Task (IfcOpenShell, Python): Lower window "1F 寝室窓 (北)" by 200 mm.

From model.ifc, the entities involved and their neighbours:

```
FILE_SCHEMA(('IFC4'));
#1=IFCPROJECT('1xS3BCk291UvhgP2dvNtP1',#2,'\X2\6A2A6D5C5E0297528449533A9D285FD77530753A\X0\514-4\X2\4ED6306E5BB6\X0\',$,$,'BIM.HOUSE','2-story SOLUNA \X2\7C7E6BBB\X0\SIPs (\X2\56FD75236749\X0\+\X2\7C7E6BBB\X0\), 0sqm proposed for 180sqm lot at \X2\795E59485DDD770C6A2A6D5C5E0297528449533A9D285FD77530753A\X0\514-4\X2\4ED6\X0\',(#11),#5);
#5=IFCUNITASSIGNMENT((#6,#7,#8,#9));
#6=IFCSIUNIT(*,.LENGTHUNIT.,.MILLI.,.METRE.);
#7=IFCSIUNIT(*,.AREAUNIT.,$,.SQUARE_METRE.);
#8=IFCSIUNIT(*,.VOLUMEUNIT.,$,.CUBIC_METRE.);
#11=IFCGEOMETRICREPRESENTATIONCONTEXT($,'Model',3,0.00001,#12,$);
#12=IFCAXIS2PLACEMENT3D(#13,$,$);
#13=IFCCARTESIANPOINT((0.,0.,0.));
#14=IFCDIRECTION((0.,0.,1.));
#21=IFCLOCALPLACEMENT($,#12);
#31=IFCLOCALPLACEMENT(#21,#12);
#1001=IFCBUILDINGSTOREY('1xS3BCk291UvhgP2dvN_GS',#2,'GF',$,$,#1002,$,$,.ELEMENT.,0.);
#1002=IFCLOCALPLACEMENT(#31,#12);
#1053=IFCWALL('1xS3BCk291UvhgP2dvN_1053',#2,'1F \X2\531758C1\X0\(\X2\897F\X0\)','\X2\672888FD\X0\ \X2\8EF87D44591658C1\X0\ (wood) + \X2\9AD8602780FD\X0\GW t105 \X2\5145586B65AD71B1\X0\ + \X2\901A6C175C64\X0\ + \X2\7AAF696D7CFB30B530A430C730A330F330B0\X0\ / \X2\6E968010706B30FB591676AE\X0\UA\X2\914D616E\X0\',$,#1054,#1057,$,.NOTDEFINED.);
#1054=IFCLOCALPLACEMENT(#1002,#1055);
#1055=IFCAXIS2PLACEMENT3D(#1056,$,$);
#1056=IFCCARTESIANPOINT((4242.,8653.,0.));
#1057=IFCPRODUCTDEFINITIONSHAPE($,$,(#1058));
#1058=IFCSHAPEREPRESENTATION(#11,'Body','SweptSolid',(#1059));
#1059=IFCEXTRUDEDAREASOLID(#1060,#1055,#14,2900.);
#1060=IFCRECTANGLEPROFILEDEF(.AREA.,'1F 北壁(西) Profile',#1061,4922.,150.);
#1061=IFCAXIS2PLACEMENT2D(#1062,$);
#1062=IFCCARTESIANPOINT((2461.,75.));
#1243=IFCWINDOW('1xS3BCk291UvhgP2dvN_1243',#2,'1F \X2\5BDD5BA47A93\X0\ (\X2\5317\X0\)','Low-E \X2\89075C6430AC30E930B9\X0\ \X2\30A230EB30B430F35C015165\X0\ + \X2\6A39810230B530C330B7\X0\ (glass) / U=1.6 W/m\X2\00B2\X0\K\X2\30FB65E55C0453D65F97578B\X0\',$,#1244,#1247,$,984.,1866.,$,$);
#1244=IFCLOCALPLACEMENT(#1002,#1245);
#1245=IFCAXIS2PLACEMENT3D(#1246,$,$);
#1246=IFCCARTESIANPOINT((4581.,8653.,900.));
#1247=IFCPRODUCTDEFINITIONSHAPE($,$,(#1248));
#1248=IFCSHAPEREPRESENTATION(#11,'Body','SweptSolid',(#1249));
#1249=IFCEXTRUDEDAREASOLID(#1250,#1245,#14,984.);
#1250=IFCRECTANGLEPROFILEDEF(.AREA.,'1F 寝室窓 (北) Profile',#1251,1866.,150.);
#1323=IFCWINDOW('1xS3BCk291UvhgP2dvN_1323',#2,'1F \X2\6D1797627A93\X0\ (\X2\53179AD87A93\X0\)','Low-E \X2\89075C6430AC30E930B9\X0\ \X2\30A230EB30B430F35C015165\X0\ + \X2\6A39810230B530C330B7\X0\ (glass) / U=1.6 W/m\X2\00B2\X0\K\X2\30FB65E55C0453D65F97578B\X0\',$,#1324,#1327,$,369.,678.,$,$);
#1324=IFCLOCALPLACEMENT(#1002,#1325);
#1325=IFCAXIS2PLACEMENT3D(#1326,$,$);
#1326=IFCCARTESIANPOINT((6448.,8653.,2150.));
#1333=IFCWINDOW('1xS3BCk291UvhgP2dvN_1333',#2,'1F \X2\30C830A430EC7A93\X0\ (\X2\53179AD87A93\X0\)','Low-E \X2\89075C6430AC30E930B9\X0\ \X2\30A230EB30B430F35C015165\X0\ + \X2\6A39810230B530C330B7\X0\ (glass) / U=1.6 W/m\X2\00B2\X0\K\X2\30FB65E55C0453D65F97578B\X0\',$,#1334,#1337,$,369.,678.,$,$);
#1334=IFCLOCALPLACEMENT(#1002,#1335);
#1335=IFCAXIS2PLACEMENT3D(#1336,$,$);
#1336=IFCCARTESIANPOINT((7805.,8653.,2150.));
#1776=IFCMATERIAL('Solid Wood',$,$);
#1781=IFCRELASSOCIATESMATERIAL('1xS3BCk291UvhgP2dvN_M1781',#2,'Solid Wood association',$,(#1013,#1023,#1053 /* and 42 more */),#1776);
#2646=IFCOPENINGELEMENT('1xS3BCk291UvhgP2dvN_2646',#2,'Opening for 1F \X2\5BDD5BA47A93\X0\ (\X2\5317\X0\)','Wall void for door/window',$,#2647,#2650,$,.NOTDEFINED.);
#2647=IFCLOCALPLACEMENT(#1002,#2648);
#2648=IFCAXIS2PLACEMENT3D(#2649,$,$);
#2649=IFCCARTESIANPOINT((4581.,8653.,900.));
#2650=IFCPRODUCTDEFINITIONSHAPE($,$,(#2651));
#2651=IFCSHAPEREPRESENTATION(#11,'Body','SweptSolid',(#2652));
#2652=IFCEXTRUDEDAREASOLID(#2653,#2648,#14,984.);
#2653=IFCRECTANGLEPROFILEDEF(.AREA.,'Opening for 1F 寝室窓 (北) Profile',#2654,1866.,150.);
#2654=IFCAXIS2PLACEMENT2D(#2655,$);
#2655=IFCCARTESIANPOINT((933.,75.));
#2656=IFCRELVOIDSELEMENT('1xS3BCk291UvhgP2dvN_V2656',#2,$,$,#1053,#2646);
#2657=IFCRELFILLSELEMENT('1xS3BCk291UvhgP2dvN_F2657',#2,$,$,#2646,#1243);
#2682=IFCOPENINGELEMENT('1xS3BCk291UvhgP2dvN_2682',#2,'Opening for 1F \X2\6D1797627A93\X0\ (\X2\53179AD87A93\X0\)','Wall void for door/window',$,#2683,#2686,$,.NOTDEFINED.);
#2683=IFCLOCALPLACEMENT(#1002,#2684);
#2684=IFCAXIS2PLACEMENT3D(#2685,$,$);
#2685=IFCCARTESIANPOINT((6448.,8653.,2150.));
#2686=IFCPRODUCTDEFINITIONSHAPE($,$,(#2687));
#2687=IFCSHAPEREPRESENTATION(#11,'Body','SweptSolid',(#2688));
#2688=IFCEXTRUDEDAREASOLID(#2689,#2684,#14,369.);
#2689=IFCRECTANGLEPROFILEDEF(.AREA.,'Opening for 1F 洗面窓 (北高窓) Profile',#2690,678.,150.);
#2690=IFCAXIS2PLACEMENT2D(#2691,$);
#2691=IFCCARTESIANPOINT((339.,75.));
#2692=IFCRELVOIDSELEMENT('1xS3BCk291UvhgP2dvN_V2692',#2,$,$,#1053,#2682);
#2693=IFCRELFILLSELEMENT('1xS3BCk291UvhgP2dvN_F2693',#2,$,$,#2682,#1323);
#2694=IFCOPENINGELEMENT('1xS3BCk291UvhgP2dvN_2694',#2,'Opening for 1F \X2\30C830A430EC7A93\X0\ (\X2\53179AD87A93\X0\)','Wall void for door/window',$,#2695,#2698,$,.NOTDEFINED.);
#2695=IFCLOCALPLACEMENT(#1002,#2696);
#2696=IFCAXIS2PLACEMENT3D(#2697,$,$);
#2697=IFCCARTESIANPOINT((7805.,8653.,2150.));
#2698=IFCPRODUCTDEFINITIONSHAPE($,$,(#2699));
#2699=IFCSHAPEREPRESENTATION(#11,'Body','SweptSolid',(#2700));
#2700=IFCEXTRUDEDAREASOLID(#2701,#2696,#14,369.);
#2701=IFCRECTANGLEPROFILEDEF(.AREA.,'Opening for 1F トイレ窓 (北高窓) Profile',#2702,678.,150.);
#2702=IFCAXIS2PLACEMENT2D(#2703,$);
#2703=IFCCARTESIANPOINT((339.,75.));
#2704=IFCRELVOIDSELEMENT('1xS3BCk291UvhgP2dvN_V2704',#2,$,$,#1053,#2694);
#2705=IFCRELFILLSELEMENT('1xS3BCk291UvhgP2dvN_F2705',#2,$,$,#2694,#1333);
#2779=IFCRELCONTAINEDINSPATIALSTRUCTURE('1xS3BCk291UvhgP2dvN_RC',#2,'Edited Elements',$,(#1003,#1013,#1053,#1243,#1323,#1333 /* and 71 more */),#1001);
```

```python
import numpy as np
import ifcopenshell
import ifcopenshell.api.geometry
import ifcopenshell.util.placement
import ifcopenshell.util.unit

model = ifcopenshell.open("model.ifc")
unit_scale = ifcopenshell.util.unit.calculate_unit_scale(model)

window = model.by_guid("1xS3BCk291UvhgP2dvN_1243")
opening = window.FillsVoids[0].RelatingOpeningElement
dz = -200.0

shift = np.array([0.0, 0.0, dz])
# The window is not placed relative to its opening, so move both.
for product in (opening, window):
    matrix = ifcopenshell.util.placement.get_local_placement(product.ObjectPlacement)
    matrix[:3, 3] += shift
    ifcopenshell.api.geometry.edit_object_placement(model, product=product, matrix=matrix, is_si=False)

print(f"moved by {dz * unit_scale:+.3f} m")

model.write("model_edited.ifc")
```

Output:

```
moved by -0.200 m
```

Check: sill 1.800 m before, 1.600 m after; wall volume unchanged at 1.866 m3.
